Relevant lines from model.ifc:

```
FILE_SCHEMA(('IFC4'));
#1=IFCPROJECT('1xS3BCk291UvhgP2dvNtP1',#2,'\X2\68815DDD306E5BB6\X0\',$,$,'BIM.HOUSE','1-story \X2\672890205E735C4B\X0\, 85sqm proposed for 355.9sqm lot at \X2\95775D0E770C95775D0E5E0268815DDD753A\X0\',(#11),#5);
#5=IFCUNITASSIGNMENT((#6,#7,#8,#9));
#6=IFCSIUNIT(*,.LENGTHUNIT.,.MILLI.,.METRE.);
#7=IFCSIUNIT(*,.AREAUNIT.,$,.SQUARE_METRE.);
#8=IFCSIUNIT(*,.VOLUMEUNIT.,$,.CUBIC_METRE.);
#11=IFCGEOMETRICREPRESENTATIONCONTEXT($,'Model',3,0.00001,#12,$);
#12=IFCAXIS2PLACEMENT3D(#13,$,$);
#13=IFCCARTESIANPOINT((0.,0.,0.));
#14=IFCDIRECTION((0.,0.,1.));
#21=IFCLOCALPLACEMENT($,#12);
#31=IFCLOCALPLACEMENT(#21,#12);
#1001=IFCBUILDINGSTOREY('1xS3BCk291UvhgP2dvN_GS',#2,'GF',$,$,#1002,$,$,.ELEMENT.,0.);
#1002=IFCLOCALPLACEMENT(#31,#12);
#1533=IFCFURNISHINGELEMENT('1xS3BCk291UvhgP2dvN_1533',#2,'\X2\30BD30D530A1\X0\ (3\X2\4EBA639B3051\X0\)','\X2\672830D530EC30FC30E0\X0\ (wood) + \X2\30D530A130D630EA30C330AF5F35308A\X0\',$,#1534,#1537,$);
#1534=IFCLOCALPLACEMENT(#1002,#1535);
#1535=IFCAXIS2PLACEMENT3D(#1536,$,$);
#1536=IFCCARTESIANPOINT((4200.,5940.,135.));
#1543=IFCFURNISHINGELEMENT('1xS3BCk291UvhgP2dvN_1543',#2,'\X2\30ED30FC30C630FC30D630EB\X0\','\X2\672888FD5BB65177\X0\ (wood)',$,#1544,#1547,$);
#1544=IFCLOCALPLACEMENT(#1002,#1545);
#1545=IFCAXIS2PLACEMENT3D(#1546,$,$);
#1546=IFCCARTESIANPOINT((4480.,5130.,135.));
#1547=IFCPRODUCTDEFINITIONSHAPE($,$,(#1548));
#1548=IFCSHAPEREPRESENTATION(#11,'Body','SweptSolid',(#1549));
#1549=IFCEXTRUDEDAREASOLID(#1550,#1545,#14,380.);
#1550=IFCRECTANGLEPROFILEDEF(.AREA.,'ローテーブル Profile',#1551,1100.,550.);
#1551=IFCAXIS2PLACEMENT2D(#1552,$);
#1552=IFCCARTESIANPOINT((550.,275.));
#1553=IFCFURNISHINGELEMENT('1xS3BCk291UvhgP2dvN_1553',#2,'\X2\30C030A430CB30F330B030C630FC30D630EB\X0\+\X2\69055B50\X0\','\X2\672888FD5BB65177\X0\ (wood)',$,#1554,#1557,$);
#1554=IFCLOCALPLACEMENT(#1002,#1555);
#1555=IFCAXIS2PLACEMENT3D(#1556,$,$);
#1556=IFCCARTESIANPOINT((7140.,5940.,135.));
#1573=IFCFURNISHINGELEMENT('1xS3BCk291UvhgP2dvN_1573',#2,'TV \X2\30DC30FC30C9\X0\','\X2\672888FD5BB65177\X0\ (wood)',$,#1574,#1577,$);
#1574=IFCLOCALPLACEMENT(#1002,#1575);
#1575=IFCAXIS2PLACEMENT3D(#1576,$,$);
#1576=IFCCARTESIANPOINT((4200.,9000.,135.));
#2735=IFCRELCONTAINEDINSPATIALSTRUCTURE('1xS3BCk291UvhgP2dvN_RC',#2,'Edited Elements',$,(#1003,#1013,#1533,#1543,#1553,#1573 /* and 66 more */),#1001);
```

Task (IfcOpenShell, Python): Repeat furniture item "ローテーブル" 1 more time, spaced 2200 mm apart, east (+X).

```python
import numpy as np
import ifcopenshell
import ifcopenshell.api.geometry
import ifcopenshell.api.root
import ifcopenshell.util.element
import ifcopenshell.util.placement
import ifcopenshell.util.unit

model = ifcopenshell.open("model.ifc")
unit_scale = ifcopenshell.util.unit.calculate_unit_scale(model)


def reuse_history(source, copy):
    """copy_class also copies each property set's owner history, people and application; keep the originals."""
    for rel in copy.IsDefinedBy:
        if rel.is_a("IfcRelDefinesByProperties") and (history := rel.RelatingPropertyDefinition.OwnerHistory):
            rel.RelatingPropertyDefinition.OwnerHistory = source.OwnerHistory
            ifcopenshell.util.element.remove_deep2(model, history)


source = model.by_id(1543)
base = ifcopenshell.util.placement.get_local_placement(source.ObjectPlacement)
step = np.array([1.0, 0.0, 0.0]) * 2.2 / unit_scale

for i in range(1, 2):
    copy = ifcopenshell.api.root.copy_class(model, product=source)
    copy.Representation = ifcopenshell.util.element.copy_deep(
        model, source.Representation, exclude=["IfcGeometricRepresentationContext", "IfcRepresentationMap"]
    )
    reuse_history(source, copy)
    matrix = base.copy()
    matrix[:3, 3] += i * step
    print("added at", matrix[:3, 3].round(3) + 0.0)
    ifcopenshell.api.geometry.edit_object_placement(model, product=copy, matrix=matrix, is_si=False)

model.write("model_edited.ifc")
```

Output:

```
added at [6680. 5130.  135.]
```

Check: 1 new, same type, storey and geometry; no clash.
